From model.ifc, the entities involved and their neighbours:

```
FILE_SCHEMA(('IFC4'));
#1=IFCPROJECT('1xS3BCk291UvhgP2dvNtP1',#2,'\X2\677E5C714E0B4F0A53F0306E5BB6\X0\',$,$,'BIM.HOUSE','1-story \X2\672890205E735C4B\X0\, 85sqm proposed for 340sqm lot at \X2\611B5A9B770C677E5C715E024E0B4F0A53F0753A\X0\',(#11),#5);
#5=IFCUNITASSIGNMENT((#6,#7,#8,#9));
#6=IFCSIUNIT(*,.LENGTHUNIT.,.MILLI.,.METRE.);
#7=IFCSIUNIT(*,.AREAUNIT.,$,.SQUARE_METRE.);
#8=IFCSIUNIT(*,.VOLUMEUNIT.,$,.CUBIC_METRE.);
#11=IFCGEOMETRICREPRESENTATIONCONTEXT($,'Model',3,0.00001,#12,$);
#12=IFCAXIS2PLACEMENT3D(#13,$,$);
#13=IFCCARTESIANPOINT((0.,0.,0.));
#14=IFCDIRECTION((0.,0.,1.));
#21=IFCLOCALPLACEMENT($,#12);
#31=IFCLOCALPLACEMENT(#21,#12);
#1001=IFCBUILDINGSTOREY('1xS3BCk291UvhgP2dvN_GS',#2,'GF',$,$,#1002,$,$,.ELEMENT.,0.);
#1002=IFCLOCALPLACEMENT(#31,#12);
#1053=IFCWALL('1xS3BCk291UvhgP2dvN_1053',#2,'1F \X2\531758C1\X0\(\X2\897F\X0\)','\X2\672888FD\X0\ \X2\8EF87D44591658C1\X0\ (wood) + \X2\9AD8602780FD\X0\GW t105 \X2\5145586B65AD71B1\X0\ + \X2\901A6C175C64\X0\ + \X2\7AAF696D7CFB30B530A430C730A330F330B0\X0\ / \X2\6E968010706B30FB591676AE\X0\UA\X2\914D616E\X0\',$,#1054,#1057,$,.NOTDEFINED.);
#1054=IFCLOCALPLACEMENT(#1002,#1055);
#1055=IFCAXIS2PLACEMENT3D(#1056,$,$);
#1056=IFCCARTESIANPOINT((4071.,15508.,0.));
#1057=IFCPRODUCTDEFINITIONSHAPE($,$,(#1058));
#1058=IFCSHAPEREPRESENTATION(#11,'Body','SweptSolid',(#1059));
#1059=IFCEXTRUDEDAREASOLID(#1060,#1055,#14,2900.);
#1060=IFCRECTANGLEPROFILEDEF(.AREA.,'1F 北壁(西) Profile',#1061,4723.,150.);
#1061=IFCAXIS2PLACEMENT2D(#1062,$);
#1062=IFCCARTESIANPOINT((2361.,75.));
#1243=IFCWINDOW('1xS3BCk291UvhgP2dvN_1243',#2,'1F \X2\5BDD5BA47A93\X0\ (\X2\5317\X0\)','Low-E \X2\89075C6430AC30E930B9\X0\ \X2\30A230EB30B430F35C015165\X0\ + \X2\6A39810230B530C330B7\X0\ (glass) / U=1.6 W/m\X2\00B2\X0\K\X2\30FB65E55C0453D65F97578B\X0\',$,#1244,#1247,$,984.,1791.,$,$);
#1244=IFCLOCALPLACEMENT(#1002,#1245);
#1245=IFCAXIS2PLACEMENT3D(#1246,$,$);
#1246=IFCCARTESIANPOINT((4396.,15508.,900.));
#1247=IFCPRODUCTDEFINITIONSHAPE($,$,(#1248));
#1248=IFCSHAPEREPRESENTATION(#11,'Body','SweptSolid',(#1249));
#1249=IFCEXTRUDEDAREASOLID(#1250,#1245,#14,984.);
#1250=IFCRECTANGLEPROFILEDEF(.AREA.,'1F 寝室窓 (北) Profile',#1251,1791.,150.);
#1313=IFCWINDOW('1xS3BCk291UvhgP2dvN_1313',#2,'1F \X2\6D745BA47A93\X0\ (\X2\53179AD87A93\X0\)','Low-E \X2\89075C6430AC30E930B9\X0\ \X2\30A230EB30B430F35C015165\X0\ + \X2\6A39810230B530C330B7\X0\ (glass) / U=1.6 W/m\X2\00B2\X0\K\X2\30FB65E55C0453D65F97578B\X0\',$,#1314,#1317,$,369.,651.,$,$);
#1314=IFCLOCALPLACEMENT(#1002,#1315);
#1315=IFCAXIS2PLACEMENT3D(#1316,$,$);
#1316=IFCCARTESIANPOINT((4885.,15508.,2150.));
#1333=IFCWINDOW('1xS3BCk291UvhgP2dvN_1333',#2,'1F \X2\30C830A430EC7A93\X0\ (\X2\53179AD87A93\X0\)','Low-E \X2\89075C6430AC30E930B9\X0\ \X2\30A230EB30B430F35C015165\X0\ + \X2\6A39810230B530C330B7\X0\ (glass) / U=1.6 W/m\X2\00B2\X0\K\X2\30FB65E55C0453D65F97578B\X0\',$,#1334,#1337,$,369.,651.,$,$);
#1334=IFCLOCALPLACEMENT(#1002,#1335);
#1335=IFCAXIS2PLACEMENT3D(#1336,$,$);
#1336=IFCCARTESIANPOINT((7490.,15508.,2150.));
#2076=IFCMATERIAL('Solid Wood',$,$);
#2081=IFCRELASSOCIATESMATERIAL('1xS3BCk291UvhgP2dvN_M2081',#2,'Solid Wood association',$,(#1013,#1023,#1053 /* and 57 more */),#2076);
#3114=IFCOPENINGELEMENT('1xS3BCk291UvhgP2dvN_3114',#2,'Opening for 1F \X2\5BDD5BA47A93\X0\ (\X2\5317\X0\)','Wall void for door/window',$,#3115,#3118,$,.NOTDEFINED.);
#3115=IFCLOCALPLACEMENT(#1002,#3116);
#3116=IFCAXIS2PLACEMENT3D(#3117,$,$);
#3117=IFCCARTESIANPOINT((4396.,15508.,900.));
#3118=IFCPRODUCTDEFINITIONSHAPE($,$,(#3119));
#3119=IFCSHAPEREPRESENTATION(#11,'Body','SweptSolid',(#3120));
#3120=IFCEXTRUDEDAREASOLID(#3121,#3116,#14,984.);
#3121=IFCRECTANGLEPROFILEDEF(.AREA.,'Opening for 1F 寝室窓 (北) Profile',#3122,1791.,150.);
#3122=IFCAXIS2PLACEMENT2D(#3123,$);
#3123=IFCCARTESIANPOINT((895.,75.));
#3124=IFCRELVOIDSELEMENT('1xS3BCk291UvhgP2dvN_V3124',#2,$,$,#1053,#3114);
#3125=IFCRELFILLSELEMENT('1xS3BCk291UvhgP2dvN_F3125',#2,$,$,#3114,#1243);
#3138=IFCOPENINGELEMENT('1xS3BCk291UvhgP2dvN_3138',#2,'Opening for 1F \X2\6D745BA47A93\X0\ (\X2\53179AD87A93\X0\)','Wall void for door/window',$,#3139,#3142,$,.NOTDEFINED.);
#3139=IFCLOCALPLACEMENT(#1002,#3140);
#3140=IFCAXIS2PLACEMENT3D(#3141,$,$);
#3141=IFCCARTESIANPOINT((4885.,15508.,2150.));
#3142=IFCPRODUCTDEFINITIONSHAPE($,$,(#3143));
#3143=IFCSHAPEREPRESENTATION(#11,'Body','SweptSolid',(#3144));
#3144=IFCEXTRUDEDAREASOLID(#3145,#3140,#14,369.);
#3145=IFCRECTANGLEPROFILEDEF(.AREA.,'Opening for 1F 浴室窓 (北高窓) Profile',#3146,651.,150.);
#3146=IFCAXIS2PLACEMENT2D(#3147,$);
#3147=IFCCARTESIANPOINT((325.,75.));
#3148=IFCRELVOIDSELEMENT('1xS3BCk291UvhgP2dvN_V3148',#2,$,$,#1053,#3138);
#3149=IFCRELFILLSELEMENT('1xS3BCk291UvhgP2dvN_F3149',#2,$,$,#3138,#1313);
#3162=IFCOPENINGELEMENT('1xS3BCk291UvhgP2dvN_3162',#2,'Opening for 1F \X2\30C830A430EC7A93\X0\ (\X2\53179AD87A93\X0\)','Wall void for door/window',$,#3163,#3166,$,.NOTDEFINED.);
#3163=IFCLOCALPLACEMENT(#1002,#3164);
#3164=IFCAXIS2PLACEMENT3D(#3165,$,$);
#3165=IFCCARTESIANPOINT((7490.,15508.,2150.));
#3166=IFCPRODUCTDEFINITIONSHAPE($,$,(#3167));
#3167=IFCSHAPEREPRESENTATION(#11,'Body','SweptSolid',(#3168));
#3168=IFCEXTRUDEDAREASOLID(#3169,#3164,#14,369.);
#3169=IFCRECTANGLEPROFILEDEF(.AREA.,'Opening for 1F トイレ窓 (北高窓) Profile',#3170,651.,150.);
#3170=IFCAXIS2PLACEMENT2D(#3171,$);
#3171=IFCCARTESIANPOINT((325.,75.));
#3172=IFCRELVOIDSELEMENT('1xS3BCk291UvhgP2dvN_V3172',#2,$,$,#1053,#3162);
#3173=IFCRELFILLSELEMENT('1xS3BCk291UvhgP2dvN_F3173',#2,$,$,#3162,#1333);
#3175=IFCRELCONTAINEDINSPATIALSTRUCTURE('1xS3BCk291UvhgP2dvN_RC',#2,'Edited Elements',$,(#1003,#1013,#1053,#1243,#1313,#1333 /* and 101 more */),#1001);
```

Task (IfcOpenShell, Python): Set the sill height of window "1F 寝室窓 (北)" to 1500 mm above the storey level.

```python
import numpy as np
import ifcopenshell
import ifcopenshell.api.geometry
import ifcopenshell.geom
import ifcopenshell.util.element
import ifcopenshell.util.placement
import ifcopenshell.util.shape
import ifcopenshell.util.unit

model = ifcopenshell.open("model.ifc")
unit_scale = ifcopenshell.util.unit.calculate_unit_scale(model)

window = model.by_guid("1xS3BCk291UvhgP2dvN_1243")
opening = window.FillsVoids[0].RelatingOpeningElement
storey = ifcopenshell.util.element.get_container(window, ifc_class="IfcBuildingStorey")
level = ifcopenshell.util.placement.get_local_placement(storey.ObjectPlacement)[2, 3]

# The opening's origin need not be at the sill, so measure its lowest point.
shape = ifcopenshell.geom.create_shape(ifcopenshell.geom.settings(), opening)
bottom = ifcopenshell.util.shape.get_shape_bottom_elevation(shape, shape.geometry) / unit_scale
dz = level + 1.5 / unit_scale - bottom

shift = np.array([0.0, 0.0, dz])
# The window is not placed relative to its opening, so move both.
for product in (opening, window):
    matrix = ifcopenshell.util.placement.get_local_placement(product.ObjectPlacement)
    matrix[:3, 3] += shift
    ifcopenshell.api.geometry.edit_object_placement(model, product=product, matrix=matrix, is_si=False)

print(f"moved by {dz * unit_scale:+.3f} m")

model.write("model_edited.ifc")
```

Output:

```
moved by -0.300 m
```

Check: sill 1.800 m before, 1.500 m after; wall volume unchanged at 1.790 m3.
